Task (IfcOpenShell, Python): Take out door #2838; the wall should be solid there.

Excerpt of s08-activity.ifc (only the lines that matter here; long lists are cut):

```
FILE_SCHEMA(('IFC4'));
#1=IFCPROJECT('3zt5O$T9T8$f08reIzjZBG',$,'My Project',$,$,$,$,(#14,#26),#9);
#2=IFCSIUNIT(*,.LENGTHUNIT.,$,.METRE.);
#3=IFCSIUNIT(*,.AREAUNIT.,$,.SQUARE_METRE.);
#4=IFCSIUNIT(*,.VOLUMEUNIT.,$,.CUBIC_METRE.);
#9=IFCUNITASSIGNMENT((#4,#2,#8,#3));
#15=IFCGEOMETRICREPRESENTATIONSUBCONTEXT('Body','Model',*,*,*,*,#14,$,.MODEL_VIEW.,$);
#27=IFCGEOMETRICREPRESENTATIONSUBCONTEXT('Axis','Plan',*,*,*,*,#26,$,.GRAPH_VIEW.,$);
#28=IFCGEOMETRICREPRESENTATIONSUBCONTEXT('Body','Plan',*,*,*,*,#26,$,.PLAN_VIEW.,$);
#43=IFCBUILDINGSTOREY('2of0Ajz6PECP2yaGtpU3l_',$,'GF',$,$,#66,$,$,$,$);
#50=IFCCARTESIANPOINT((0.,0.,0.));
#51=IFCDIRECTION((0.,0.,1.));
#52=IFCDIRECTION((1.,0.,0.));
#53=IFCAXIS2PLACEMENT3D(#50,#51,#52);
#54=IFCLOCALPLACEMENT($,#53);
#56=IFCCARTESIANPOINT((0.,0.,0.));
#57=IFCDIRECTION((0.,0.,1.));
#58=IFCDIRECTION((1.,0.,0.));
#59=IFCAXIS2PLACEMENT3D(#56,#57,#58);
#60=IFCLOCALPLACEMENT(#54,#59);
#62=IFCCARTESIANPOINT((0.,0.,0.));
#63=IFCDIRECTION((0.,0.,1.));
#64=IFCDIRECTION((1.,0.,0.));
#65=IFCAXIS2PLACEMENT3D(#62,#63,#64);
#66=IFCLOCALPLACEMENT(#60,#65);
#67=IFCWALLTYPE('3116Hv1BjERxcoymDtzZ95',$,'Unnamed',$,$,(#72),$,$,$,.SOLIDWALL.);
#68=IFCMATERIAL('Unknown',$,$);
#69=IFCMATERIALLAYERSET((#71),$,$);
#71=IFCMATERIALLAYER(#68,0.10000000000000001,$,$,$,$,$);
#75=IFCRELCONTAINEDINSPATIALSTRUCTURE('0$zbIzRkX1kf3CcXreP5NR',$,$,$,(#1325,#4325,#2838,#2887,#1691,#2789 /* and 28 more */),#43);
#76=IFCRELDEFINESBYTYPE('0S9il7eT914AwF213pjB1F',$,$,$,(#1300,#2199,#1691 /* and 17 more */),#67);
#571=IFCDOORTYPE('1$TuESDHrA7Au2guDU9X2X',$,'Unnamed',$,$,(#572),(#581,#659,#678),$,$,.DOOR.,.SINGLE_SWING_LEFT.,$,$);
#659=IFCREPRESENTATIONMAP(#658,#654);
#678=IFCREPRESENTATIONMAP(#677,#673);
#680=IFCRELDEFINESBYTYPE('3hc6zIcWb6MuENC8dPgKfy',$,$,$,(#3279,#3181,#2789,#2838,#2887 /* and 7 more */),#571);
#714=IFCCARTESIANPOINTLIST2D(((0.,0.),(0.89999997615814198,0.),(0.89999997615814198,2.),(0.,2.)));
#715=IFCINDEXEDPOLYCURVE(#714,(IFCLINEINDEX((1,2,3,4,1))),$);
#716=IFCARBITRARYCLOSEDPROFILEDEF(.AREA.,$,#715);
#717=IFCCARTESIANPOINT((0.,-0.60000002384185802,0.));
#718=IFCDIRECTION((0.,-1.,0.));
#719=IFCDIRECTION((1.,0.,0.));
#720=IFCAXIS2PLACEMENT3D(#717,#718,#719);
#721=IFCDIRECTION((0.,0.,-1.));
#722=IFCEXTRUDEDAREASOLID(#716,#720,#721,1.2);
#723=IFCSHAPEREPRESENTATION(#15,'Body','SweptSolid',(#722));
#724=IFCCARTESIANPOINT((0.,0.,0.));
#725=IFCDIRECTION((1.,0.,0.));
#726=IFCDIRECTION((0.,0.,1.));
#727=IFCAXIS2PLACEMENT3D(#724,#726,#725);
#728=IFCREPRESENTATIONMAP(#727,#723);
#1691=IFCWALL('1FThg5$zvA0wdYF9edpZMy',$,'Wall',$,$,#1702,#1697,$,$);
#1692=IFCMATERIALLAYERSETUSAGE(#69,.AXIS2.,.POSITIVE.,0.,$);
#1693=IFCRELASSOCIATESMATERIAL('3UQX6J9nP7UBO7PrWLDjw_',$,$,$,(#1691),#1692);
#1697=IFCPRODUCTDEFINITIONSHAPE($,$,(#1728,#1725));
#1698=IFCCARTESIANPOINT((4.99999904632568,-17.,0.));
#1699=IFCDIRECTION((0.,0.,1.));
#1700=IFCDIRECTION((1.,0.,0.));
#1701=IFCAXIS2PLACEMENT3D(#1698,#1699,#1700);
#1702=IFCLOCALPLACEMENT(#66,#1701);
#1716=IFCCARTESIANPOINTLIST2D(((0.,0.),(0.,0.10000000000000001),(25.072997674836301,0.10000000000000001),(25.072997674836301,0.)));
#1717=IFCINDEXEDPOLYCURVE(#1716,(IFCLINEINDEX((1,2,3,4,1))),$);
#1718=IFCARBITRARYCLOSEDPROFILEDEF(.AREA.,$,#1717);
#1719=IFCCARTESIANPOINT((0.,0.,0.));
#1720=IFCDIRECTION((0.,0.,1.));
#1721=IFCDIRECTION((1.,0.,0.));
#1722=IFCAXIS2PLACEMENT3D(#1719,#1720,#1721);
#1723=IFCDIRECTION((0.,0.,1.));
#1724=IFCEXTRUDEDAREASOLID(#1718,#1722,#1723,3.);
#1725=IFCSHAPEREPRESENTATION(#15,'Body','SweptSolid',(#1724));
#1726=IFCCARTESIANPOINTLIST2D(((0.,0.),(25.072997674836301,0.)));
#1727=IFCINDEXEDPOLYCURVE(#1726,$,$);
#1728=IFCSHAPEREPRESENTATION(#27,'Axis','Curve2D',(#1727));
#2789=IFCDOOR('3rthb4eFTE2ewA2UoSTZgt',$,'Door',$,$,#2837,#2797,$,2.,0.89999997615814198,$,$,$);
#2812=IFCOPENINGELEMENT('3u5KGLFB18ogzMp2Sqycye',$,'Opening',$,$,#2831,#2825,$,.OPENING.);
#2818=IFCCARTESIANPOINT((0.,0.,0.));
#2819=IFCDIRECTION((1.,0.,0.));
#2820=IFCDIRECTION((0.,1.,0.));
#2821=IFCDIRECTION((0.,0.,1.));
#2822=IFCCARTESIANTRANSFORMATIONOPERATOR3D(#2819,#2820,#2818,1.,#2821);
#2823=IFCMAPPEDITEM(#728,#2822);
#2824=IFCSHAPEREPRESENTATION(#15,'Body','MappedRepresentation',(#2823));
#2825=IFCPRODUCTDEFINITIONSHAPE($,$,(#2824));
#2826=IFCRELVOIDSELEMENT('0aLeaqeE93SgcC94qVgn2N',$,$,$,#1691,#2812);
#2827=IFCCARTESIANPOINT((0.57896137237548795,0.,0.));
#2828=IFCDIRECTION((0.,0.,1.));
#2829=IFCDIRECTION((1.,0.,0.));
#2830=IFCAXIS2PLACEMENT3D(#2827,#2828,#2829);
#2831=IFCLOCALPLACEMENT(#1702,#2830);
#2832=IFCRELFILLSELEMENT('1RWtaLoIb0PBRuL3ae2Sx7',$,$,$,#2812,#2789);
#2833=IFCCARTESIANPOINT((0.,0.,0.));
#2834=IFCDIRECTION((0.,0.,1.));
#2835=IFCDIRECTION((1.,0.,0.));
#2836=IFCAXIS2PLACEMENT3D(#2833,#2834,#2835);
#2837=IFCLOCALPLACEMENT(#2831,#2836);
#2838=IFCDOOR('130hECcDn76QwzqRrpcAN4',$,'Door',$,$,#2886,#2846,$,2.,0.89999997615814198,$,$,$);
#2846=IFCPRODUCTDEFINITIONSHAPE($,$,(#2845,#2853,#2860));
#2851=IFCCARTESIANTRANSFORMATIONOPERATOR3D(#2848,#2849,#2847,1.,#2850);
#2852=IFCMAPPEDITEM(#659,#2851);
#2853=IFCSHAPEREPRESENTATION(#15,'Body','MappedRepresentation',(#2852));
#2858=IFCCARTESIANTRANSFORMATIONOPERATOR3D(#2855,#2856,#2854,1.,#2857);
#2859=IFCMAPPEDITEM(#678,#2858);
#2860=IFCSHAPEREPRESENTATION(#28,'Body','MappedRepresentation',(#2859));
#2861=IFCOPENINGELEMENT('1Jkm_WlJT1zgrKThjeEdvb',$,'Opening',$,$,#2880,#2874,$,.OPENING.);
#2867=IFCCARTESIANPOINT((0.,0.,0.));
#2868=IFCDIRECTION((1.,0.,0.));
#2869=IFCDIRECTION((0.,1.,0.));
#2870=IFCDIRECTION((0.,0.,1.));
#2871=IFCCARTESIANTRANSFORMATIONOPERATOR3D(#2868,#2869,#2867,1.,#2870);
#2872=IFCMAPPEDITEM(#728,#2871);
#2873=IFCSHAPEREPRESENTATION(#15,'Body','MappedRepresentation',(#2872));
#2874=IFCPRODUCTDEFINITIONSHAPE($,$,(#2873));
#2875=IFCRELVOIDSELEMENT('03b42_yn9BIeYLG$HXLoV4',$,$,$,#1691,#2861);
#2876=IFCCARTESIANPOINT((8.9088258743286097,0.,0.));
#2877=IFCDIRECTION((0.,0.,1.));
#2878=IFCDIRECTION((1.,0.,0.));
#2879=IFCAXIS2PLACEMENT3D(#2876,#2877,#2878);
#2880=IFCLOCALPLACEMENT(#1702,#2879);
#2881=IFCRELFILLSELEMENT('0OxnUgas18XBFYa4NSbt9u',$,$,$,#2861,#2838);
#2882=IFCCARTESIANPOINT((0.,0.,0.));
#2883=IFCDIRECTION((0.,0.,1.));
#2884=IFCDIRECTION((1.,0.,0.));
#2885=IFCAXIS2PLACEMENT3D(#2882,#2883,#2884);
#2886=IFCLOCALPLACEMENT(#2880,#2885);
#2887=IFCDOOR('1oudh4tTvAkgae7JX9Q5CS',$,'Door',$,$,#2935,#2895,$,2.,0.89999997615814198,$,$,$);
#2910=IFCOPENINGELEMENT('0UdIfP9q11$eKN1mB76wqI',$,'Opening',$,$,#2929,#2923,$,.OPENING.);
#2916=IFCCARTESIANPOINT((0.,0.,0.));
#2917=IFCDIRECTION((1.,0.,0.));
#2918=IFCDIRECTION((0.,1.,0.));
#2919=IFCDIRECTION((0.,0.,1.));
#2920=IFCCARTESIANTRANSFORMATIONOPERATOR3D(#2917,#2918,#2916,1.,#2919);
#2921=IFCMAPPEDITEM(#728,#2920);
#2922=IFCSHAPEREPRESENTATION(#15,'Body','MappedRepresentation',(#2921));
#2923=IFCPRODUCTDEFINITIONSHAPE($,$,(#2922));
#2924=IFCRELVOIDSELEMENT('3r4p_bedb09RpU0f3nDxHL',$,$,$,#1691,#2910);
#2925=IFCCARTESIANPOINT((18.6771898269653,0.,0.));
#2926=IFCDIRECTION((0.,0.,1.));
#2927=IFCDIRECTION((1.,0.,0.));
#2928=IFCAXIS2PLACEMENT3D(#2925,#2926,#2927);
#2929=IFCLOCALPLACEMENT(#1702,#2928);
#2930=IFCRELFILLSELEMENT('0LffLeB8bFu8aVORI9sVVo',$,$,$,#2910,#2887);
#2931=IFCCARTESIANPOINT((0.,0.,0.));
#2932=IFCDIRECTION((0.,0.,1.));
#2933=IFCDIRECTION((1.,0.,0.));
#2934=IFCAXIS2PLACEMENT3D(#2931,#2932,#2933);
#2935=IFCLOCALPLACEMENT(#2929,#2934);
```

```python
import ifcopenshell
import ifcopenshell.api.feature
import ifcopenshell.api.root
import ifcopenshell.geom
import ifcopenshell.util.shape

model = ifcopenshell.open("s08-activity.ifc")
settings = ifcopenshell.geom.settings()


def volume(element):
    """Net volume in cubic metres, openings subtracted."""
    shape = ifcopenshell.geom.create_shape(settings, element)
    return ifcopenshell.util.shape.get_volume(shape.geometry)


door = model.by_guid("130hECcDn76QwzqRrpcAN4")
opening = door.FillsVoids[0].RelatingOpeningElement
wall = opening.VoidsElements[0].RelatingBuildingElement
before = volume(wall)

ifcopenshell.api.root.remove_product(model, product=door)
ifcopenshell.api.feature.remove_feature(model, feature=opening)

after = volume(wall)

print(f"wall volume {before:.3f} -> {after:.3f} m3")

model.write("s08-activity_rev.ifc")
```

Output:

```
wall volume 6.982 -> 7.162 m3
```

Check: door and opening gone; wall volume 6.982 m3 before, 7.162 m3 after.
